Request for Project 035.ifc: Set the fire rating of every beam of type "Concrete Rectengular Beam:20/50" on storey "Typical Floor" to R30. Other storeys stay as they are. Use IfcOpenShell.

First a look at what the model holds.

```python
import ifcopenshell
import ifcopenshell.util.element

model = ifcopenshell.open("Project 035.ifc")
print(model.schema)
storey = next(s for s in model.by_type("IfcBuildingStorey") if s.Name == "Typical Floor")
beams = [e for e in ifcopenshell.util.element.get_decomposition(storey) if e.is_a("IfcBeam")]
seen = {}
for e in beams:
    element_type = ifcopenshell.util.element.get_type(e)
    key = (element_type.Name if element_type != e and element_type else None, ifcopenshell.util.element.get_pset(e, "Pset_BeamCommon", "FireRating"))
    seen[key] = seen.get(key, 0) + 1
for (name, value), count in sorted(seen.items(), key=str):
    print(count, "x", name, "|", value)
```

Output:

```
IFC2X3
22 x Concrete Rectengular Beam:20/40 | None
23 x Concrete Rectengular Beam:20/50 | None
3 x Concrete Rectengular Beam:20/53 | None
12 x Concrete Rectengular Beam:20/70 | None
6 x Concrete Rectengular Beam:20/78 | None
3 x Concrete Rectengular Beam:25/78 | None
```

```python
import ifcopenshell
import ifcopenshell.api.pset
import ifcopenshell.util.element

model = ifcopenshell.open("Project 035.ifc")

storey = next(s for s in model.by_type("IfcBuildingStorey") if s.Name == "Typical Floor")
beams = [e for e in ifcopenshell.util.element.get_decomposition(storey) if e.is_a("IfcBeam")]

count = 0
for e in beams:
    element_type = ifcopenshell.util.element.get_type(e)
    if element_type in (None, e) or element_type.Name != "Concrete Rectengular Beam:20/50":
        continue
    # add_pset returns the element's existing set when there is one.
    pset = ifcopenshell.api.pset.add_pset(model, product=e, name="Pset_BeamCommon")
    ifcopenshell.api.pset.edit_pset(model, pset=pset, properties={"FireRating": "R30"})
    count += 1

print(count, "beams updated")

model.write("Project 035_edited.ifc")
```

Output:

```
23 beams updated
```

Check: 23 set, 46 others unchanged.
